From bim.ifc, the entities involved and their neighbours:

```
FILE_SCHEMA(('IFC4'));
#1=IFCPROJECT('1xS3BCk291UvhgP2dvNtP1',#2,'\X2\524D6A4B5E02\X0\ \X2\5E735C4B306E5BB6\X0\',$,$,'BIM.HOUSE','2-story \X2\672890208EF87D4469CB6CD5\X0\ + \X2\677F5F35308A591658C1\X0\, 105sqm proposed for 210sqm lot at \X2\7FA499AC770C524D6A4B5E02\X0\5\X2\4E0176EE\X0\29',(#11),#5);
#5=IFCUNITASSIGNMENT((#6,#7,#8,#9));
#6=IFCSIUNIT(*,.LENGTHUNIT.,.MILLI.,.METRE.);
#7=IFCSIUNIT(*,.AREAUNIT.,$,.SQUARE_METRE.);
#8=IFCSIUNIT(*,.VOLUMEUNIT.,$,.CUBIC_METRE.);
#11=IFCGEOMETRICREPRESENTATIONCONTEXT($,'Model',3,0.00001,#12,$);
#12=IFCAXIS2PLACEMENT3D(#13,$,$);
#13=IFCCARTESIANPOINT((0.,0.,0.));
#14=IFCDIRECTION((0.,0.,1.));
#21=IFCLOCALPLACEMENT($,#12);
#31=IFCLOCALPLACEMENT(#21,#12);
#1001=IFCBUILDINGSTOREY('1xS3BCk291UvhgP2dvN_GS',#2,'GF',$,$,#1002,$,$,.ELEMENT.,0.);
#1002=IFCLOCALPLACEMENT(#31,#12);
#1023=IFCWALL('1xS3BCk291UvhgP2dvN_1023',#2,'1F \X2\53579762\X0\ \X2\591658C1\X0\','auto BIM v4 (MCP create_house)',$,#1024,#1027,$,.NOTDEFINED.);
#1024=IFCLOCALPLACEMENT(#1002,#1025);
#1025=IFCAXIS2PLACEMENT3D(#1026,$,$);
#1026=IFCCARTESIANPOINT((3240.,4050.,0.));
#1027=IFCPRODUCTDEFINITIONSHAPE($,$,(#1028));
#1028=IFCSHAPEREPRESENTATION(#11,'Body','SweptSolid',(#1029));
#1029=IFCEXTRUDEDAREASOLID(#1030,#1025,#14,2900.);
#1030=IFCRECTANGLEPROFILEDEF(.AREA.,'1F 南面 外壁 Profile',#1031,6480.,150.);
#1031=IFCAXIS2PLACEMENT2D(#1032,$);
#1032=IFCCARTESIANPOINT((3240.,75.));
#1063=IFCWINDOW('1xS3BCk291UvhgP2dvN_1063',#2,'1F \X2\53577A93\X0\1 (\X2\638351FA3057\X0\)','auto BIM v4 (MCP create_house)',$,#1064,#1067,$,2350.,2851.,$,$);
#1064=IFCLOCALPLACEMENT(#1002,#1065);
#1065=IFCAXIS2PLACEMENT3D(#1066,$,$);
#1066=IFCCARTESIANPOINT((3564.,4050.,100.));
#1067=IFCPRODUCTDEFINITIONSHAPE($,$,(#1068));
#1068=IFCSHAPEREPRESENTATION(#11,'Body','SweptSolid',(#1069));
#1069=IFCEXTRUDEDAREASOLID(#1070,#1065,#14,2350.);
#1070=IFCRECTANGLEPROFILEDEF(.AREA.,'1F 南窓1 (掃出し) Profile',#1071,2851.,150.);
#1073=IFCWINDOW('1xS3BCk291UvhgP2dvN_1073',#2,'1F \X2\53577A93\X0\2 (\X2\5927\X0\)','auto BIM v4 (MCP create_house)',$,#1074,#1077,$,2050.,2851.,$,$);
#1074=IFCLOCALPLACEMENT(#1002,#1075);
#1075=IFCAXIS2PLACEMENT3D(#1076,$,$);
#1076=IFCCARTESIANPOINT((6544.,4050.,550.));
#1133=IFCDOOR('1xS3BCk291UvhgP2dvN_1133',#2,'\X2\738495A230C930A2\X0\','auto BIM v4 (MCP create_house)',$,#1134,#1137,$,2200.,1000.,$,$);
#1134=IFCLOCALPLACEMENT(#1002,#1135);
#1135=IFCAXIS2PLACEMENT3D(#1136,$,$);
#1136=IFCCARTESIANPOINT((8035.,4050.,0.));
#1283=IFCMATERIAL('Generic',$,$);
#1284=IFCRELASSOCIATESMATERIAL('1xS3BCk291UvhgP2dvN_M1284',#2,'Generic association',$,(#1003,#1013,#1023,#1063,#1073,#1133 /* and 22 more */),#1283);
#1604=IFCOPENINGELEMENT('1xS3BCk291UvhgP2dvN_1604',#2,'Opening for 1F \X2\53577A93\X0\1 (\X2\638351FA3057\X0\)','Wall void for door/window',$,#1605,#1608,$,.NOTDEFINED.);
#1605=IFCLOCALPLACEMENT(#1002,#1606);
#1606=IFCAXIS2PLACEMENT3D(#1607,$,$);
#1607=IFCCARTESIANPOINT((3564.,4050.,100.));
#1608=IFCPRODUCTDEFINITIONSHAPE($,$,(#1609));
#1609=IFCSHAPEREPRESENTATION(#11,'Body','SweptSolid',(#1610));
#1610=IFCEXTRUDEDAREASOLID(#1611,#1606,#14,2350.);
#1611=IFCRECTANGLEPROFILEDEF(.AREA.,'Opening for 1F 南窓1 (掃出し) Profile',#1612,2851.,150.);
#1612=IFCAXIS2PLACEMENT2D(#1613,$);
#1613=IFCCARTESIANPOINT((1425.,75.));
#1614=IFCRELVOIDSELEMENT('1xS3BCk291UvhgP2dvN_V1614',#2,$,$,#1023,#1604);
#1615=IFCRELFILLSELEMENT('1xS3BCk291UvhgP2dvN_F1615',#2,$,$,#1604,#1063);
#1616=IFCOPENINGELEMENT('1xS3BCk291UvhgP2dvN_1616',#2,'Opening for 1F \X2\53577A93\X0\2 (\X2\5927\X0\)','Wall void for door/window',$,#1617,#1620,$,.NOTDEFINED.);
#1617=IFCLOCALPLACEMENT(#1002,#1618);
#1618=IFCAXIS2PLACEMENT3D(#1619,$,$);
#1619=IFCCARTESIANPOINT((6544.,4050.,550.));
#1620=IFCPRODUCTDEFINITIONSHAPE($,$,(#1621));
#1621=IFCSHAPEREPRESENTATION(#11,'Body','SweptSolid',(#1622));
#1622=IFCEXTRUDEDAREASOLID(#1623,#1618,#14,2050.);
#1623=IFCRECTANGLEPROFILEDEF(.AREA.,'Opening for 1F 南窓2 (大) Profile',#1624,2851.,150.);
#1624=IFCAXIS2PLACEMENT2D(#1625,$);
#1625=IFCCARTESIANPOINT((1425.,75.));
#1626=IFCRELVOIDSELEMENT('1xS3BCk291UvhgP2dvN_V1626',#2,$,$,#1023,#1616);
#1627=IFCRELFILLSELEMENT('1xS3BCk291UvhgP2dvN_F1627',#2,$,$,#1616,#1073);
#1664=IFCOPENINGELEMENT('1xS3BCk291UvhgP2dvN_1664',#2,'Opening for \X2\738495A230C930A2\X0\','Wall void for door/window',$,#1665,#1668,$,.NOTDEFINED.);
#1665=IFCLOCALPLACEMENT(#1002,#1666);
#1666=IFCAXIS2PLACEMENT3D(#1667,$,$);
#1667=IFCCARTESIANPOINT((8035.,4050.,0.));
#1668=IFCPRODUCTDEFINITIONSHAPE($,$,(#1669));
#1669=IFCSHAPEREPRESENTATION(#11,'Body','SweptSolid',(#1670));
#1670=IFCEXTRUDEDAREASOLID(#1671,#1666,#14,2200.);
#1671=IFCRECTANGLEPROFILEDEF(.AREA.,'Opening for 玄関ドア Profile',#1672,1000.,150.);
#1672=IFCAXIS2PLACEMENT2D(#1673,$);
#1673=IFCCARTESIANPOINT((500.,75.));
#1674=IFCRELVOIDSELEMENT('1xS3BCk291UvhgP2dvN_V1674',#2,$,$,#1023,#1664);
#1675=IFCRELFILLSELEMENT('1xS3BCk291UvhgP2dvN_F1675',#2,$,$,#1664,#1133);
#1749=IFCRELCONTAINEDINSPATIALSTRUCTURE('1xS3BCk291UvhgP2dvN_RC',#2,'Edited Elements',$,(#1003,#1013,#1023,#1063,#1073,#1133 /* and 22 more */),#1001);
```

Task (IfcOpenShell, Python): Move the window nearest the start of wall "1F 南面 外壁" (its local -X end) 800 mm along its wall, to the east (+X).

```python
import ifcopenshell
import ifcopenshell.api.geometry
import ifcopenshell.util.placement

model = ifcopenshell.open("bim.ifc")

window = model.by_id(1063)
opening = window.FillsVoids[0].RelatingOpeningElement
wall = opening.VoidsElements[0].RelatingBuildingElement

wall_matrix = ifcopenshell.util.placement.get_local_placement(wall.ObjectPlacement)
shift = wall_matrix[:3, 0] * 800.0
before = ifcopenshell.util.placement.get_local_placement(window.ObjectPlacement)[:3, 3].copy()

# The window is not placed relative to its opening, so move both.
for product in (opening, window):
    matrix = ifcopenshell.util.placement.get_local_placement(product.ObjectPlacement)
    matrix[:3, 3] += shift
    ifcopenshell.api.geometry.edit_object_placement(model, product=product, matrix=matrix, is_si=False)

after = ifcopenshell.util.placement.get_local_placement(window.ObjectPlacement)[:3, 3]
print("window moved by", (after - before).round(3) + 0.0)

model.write("bim_updated.ifc")
```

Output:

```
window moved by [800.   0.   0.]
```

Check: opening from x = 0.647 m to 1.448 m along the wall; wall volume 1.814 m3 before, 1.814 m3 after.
